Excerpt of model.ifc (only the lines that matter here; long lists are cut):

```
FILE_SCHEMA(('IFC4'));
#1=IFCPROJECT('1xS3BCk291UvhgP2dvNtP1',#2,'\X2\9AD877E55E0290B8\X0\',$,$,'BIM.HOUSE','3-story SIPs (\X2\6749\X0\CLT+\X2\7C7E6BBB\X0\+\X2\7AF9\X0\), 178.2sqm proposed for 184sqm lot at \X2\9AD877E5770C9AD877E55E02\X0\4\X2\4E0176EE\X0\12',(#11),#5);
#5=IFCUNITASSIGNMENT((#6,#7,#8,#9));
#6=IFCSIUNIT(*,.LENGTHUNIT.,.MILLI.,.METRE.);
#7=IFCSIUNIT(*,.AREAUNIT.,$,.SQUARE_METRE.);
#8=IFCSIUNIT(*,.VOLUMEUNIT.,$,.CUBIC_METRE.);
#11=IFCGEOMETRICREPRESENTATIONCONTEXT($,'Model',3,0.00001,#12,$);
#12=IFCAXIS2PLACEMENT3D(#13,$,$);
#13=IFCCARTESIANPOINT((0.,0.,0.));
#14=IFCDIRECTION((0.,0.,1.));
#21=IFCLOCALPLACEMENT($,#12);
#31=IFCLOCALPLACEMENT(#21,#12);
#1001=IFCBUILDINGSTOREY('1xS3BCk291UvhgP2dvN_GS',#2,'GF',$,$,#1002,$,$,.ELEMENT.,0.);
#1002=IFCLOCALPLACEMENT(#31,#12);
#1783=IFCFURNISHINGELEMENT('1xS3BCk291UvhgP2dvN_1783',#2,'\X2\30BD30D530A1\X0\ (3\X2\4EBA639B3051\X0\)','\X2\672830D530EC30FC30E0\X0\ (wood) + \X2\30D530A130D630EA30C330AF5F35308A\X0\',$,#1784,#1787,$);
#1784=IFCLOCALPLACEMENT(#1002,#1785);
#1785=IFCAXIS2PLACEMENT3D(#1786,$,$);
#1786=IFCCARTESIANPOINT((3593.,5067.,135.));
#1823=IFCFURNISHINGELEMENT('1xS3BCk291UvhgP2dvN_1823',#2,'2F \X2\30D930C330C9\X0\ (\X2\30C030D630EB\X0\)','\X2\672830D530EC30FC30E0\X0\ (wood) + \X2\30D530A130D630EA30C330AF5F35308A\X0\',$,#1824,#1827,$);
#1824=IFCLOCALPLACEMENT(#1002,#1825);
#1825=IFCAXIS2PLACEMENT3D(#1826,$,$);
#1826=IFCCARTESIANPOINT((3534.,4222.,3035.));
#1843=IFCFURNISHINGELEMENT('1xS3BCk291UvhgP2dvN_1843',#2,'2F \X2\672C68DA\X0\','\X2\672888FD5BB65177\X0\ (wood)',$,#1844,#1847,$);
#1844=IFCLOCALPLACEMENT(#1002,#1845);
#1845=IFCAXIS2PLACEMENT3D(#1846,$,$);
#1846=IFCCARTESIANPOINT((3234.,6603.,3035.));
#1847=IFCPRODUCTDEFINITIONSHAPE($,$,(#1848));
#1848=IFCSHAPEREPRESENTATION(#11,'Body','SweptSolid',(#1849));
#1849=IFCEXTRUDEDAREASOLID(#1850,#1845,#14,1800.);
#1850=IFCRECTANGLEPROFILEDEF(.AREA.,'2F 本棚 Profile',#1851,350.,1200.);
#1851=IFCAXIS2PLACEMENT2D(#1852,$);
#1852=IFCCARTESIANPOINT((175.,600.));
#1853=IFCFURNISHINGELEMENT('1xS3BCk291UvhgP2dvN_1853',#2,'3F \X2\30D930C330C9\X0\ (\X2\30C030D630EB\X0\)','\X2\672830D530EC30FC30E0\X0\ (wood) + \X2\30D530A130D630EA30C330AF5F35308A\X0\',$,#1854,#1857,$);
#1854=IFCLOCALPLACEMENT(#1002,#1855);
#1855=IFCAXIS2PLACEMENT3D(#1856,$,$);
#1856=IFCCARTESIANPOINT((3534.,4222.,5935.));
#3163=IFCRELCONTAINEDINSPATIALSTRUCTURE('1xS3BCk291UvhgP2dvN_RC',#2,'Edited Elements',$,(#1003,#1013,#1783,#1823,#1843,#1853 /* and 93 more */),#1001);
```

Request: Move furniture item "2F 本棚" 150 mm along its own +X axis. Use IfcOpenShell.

```python
import ifcopenshell
import ifcopenshell.api.geometry
import ifcopenshell.util.placement
import ifcopenshell.util.unit

model = ifcopenshell.open("model.ifc")
unit_scale = ifcopenshell.util.unit.calculate_unit_scale(model)

item = model.by_guid("1xS3BCk291UvhgP2dvN_1843")
matrix = ifcopenshell.util.placement.get_local_placement(item.ObjectPlacement)
matrix[:3, 3] += matrix[:3, 0] * 0.15 / unit_scale
ifcopenshell.api.geometry.edit_object_placement(model, product=item, matrix=matrix, is_si=False)

print(ifcopenshell.util.placement.get_local_placement(item.ObjectPlacement).round(3) + 0.0)

model.write("model_rev.ifc")
```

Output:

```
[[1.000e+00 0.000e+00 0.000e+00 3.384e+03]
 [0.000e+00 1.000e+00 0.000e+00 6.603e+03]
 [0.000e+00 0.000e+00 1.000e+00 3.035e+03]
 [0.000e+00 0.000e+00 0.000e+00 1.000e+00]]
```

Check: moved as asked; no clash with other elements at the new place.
